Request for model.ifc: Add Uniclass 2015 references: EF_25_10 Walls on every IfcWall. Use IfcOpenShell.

First a look at what the model holds.

```python
import ifcopenshell

model = ifcopenshell.open("model.ifc")
print(model.schema)
print("classifications:", [c.Name for c in model.by_type("IfcClassification")])
for ifc_class in ("IfcDoor", "IfcRoof", "IfcStair", "IfcWall", "IfcWindow"):
    print(ifc_class, len(model.by_type(ifc_class)))
```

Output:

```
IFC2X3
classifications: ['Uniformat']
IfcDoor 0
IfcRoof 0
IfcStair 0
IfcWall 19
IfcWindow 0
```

```python
import ifcopenshell
import ifcopenshell.api.classification

model = ifcopenshell.open("model.ifc")

# IFC2X3 requires Source and Edition and has no link from the project to the system.
system = model.create_entity("IfcClassification", Source="NBS", Edition="2015", Name="Uniclass 2015")

codes = {
    "IfcWall": ("EF_25_10", "Walls"),
}
for ifc_class, (code, name) in codes.items():
    products = model.by_type(ifc_class)
    ifcopenshell.api.classification.add_reference(
        model, products=products, classification=system, identification=code, name=name
    )
    print(code, len(products))

model.write("model_v2.ifc")
```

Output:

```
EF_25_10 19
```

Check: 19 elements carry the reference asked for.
